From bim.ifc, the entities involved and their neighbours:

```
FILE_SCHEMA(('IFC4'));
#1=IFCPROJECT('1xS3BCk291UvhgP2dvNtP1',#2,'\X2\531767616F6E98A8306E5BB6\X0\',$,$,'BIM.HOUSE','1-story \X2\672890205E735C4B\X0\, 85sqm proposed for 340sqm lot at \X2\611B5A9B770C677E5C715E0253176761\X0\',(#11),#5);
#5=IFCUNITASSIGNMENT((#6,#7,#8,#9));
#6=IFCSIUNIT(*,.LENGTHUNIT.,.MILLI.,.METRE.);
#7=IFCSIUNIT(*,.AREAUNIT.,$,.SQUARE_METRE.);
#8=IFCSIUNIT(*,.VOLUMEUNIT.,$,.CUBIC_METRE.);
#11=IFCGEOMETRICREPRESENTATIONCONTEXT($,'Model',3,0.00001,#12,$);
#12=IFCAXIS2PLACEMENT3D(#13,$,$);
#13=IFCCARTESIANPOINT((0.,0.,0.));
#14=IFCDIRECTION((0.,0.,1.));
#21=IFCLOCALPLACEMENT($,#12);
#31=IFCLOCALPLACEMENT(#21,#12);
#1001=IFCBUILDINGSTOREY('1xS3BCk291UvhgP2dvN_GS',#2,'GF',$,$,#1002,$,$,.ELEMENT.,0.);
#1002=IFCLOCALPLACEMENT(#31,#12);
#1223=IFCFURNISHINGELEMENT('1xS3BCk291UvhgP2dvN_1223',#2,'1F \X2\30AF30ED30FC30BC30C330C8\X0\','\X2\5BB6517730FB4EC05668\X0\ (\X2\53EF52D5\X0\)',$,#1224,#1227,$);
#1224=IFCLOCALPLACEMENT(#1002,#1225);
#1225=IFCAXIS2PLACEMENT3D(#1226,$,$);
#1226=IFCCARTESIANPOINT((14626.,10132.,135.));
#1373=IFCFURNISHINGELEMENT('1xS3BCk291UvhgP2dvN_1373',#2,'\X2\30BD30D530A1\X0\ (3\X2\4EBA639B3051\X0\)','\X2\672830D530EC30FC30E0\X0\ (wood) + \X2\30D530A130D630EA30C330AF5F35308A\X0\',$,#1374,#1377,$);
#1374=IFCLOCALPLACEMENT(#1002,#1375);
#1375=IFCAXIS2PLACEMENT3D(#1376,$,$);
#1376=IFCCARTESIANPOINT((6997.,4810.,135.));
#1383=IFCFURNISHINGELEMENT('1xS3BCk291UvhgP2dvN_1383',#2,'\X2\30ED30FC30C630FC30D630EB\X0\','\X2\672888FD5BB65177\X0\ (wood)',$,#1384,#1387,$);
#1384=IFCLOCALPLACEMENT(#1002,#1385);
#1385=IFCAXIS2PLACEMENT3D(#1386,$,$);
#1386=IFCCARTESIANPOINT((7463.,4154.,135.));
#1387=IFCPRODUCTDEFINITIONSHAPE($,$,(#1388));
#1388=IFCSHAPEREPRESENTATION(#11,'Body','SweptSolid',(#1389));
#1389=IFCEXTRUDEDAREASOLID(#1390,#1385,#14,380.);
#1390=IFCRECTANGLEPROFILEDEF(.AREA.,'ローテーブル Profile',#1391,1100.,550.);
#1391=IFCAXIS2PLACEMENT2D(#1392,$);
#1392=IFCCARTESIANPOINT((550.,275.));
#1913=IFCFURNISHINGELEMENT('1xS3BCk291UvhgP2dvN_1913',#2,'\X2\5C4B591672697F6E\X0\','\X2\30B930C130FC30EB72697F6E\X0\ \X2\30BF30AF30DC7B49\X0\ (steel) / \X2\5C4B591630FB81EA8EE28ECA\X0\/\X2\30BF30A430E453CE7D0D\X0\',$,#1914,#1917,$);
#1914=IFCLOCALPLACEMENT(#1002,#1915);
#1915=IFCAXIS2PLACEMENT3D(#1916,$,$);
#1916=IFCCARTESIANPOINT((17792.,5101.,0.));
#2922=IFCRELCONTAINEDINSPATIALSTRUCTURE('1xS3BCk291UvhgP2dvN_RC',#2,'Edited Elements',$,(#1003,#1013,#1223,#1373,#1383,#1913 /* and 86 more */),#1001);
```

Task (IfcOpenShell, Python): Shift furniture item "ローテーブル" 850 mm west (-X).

```python
import ifcopenshell
import ifcopenshell.api.geometry
import ifcopenshell.util.placement

model = ifcopenshell.open("bim.ifc")

item = model.by_guid("1xS3BCk291UvhgP2dvN_1383")
matrix = ifcopenshell.util.placement.get_local_placement(item.ObjectPlacement)
matrix[0, 3] -= 850.0
ifcopenshell.api.geometry.edit_object_placement(model, product=item, matrix=matrix, is_si=False)

print(ifcopenshell.util.placement.get_local_placement(item.ObjectPlacement).round(3) + 0.0)

model.write("bim_v2.ifc")
```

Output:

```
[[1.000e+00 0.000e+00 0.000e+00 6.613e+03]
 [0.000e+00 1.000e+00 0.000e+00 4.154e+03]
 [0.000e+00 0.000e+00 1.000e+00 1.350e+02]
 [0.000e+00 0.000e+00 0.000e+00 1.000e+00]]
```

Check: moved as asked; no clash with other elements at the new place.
